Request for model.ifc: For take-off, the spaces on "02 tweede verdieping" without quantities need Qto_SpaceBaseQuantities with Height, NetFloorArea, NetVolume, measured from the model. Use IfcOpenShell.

First a look at what the model holds.

```python
import ifcopenshell
import ifcopenshell.util.element
import ifcopenshell.util.unit

model = ifcopenshell.open("model.ifc")
print(model.schema)
for unit_type in ("LENGTHUNIT", "AREAUNIT", "VOLUMEUNIT"):
    print(unit_type, ifcopenshell.util.unit.calculate_unit_scale(model, unit_type))
storey = next(s for s in model.by_type("IfcBuildingStorey") if s.Name == "02 tweede verdieping")
spaces = [e for e in ifcopenshell.util.element.get_decomposition(storey) if e.is_a("IfcSpace")]
for e in sorted(spaces, key=lambda e: e.id()):
    print(e.id(), e.is_a(), e.Name, list(ifcopenshell.util.element.get_psets(e, qtos_only=True)), sep=" | ")
```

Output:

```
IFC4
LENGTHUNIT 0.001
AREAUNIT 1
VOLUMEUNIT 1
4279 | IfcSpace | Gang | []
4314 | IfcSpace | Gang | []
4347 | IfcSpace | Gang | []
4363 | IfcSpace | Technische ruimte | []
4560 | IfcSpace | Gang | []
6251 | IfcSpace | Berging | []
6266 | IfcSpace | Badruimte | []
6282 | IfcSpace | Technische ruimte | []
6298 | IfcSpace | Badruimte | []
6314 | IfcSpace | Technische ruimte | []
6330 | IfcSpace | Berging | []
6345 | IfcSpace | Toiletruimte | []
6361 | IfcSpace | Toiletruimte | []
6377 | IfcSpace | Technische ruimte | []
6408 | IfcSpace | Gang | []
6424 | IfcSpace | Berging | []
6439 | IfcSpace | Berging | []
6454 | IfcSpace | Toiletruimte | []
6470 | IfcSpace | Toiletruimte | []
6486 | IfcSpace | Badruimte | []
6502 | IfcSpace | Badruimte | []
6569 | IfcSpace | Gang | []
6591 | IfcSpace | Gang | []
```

```python
import ifcopenshell
import ifcopenshell.api.pset
import ifcopenshell.geom
import ifcopenshell.util.element
import ifcopenshell.util.shape
import ifcopenshell.util.unit

model = ifcopenshell.open("model.ifc")
unit_scale = ifcopenshell.util.unit.calculate_unit_scale(model)
area_scale = ifcopenshell.util.unit.calculate_unit_scale(model, "AREAUNIT")
volume_scale = ifcopenshell.util.unit.calculate_unit_scale(model, "VOLUMEUNIT")
settings = ifcopenshell.geom.settings()

storey = next(s for s in model.by_type("IfcBuildingStorey") if s.Name == "02 tweede verdieping")
spaces = [e for e in ifcopenshell.util.element.get_decomposition(storey) if e.is_a("IfcSpace")]

for e in sorted(spaces, key=lambda e: e.id()):
    if ifcopenshell.util.element.get_psets(e, qtos_only=True, should_inherit=False):
        continue
    # Geometry comes back in metres, in the element's own axes.
    shape = ifcopenshell.geom.create_shape(settings, e)
    values = {
        "Height": ifcopenshell.util.shape.get_z(shape.geometry) / unit_scale,
        "NetFloorArea": ifcopenshell.util.shape.get_footprint_area(shape.geometry) / area_scale,
        "NetVolume": ifcopenshell.util.shape.get_volume(shape.geometry) / volume_scale,
    }
    qto = ifcopenshell.api.pset.add_qto(model, product=e, name="Qto_SpaceBaseQuantities")
    ifcopenshell.api.pset.edit_qto(model, qto=qto, properties=values)
    print(e.id(), {k: round(v, 3) for k, v in values.items()})

model.write("model_rev.ifc")
```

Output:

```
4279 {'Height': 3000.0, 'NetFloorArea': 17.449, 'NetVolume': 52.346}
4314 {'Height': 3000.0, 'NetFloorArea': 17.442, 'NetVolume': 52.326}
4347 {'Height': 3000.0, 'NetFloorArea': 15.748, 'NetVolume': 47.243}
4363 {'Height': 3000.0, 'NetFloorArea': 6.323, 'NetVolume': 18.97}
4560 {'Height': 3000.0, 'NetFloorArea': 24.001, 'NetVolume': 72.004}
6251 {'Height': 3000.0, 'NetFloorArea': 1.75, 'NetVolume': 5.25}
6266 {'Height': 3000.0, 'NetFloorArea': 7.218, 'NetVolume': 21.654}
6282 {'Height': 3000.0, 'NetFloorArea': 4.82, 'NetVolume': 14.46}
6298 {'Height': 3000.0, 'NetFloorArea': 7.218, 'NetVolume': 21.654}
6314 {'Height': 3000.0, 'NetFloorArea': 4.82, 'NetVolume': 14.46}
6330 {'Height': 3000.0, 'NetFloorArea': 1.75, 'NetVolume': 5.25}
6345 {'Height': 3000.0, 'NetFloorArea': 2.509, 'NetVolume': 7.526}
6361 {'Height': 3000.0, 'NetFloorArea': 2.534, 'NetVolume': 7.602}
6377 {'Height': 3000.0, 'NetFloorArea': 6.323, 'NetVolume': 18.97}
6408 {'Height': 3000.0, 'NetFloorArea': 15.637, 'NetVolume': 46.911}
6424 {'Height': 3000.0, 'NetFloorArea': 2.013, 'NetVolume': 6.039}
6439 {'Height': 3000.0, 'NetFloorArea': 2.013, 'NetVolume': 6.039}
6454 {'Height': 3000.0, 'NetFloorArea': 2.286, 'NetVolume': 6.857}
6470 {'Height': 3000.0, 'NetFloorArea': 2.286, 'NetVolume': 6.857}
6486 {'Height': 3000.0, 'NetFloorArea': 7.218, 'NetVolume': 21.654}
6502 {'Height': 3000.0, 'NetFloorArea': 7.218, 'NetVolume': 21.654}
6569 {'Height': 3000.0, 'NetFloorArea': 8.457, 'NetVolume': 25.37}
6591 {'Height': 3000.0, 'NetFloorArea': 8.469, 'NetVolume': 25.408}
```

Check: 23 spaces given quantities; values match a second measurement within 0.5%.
